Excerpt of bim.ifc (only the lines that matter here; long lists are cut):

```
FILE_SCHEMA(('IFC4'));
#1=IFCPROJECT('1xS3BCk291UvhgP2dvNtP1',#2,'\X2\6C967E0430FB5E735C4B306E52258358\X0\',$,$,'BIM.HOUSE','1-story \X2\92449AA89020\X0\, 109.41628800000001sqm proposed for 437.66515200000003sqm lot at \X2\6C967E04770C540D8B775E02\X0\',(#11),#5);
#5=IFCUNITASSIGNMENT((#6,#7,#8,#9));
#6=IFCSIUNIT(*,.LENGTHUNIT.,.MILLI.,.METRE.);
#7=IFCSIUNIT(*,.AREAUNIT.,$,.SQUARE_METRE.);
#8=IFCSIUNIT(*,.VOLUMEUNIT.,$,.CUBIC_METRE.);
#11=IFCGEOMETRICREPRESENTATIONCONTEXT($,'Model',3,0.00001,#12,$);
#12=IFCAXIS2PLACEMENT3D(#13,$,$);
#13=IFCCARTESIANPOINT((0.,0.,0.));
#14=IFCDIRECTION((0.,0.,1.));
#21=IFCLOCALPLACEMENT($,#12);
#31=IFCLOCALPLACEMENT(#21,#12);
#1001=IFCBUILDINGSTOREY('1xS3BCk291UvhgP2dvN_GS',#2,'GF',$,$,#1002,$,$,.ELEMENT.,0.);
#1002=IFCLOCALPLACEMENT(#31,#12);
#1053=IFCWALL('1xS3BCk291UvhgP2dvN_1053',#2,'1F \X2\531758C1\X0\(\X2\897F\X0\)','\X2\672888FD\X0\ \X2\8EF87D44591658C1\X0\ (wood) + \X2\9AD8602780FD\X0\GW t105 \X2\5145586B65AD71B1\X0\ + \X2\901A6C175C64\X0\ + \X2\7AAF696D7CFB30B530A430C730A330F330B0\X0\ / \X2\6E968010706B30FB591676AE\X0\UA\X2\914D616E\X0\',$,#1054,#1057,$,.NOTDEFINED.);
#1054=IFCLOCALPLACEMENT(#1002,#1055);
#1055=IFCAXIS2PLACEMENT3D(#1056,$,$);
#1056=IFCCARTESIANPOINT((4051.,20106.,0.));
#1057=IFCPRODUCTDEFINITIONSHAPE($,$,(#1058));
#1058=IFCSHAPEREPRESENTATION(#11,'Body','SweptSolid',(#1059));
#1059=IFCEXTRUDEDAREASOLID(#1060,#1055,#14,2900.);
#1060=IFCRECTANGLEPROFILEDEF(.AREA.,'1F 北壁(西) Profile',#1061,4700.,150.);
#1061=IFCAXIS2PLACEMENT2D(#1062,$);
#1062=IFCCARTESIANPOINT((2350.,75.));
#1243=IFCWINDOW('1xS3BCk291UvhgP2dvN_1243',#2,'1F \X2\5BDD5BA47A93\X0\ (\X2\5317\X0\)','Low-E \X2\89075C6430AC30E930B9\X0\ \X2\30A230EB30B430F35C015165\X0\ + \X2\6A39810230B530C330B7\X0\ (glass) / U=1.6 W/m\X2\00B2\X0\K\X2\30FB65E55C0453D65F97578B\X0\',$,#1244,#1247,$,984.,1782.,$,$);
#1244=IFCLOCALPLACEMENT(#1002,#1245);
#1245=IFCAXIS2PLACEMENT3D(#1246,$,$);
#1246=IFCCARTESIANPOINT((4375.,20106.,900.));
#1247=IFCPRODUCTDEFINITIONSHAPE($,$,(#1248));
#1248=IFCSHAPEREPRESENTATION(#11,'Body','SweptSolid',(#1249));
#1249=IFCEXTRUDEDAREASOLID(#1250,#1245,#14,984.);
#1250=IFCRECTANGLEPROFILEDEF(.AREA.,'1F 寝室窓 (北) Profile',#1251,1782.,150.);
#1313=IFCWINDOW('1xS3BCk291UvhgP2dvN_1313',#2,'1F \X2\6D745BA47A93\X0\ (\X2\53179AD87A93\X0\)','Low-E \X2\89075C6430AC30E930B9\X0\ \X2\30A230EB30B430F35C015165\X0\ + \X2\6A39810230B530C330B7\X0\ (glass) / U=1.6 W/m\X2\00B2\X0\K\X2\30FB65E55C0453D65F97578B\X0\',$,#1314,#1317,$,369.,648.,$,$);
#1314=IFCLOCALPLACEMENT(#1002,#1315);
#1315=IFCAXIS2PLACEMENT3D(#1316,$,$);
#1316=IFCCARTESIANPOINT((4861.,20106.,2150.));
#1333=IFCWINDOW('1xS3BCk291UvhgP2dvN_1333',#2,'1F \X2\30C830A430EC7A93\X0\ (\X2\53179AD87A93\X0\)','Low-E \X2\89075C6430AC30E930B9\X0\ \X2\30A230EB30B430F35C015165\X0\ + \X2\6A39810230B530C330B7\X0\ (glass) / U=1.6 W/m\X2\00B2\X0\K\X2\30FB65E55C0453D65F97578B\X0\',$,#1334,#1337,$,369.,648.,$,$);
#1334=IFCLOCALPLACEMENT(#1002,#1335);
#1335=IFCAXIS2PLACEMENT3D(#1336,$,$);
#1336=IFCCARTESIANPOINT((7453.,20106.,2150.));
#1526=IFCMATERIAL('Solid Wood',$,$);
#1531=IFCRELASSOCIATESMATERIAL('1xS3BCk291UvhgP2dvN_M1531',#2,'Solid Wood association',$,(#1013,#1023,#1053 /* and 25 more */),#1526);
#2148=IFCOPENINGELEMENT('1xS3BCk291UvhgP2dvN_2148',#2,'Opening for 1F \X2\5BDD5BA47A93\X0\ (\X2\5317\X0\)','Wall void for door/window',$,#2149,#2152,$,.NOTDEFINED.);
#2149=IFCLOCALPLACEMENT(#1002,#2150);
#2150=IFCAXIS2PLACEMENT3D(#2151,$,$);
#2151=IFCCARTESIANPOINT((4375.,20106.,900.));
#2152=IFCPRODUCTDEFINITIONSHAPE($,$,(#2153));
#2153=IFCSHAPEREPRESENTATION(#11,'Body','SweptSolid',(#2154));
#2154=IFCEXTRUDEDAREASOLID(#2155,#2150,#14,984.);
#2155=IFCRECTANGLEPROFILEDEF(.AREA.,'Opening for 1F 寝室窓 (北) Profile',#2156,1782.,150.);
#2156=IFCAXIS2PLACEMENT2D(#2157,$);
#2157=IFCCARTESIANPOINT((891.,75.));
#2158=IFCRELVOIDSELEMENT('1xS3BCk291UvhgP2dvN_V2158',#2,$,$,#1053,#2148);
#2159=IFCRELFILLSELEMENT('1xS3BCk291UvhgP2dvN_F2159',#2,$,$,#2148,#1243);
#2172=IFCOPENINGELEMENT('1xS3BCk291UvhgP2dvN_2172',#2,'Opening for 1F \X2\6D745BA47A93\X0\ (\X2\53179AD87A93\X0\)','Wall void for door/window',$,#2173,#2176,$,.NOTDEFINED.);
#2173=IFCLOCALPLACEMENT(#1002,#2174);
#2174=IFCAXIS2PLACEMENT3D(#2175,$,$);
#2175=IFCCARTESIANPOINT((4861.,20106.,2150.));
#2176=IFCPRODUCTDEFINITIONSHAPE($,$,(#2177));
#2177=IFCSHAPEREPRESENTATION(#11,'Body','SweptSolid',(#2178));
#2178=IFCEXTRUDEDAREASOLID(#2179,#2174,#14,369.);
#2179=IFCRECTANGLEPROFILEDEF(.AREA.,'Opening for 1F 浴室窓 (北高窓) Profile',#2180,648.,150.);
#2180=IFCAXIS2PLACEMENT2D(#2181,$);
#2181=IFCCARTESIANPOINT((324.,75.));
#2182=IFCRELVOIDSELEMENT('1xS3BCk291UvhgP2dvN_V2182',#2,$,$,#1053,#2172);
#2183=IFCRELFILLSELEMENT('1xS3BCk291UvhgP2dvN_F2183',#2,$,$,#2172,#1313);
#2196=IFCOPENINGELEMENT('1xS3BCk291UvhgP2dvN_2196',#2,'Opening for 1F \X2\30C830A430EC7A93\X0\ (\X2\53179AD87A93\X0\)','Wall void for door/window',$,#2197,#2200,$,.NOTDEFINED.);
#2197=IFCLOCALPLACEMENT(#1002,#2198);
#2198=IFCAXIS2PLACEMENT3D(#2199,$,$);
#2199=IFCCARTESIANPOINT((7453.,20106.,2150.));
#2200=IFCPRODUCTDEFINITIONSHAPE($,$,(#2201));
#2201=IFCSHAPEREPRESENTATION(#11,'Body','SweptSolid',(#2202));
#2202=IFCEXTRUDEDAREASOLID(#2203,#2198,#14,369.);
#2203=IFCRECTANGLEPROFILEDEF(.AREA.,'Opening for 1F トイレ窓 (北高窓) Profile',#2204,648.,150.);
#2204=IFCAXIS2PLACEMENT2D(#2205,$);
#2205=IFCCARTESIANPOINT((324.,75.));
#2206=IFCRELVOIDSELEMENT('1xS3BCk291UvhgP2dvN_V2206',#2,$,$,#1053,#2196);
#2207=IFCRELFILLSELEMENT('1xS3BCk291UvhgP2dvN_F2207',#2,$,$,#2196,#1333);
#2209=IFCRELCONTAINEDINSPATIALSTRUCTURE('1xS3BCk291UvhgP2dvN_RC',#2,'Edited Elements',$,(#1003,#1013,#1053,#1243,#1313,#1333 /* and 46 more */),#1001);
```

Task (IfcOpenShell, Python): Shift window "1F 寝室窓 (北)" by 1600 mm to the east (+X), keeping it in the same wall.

```python
import ifcopenshell
import ifcopenshell.api.geometry
import ifcopenshell.util.placement

model = ifcopenshell.open("bim.ifc")

window = model.by_guid("1xS3BCk291UvhgP2dvN_1243")
opening = window.FillsVoids[0].RelatingOpeningElement
wall = opening.VoidsElements[0].RelatingBuildingElement

wall_matrix = ifcopenshell.util.placement.get_local_placement(wall.ObjectPlacement)
shift = wall_matrix[:3, 0] * 1600.0
before = ifcopenshell.util.placement.get_local_placement(window.ObjectPlacement)[:3, 3].copy()

# The window is not placed relative to its opening, so move both.
for product in (opening, window):
    matrix = ifcopenshell.util.placement.get_local_placement(product.ObjectPlacement)
    matrix[:3, 3] += shift
    ifcopenshell.api.geometry.edit_object_placement(model, product=product, matrix=matrix, is_si=False)

after = ifcopenshell.util.placement.get_local_placement(window.ObjectPlacement)[:3, 3]
print("window moved by", (after - before).round(3) + 0.0)

model.write("bim-out.ifc")
```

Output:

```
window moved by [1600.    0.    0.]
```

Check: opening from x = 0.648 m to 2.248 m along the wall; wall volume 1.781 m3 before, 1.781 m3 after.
